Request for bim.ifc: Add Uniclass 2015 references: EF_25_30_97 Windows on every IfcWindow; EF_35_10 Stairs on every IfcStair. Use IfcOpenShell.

First a look at what the model holds.

```python
import ifcopenshell

model = ifcopenshell.open("bim.ifc")
print(model.schema)
print("classifications:", [c.Name for c in model.by_type("IfcClassification")])
for ifc_class in ("IfcDoor", "IfcRoof", "IfcStair", "IfcWall", "IfcWindow"):
    print(ifc_class, len(model.by_type(ifc_class)))
```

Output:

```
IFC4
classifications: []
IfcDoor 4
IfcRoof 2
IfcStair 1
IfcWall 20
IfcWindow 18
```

```python
import ifcopenshell
import ifcopenshell.api.classification

model = ifcopenshell.open("bim.ifc")

system = ifcopenshell.api.classification.add_classification(model, classification="Uniclass 2015")

codes = {
    "IfcWindow": ("EF_25_30_97", "Windows"),
    "IfcStair": ("EF_35_10", "Stairs"),
}
for ifc_class, (code, name) in codes.items():
    products = model.by_type(ifc_class)
    ifcopenshell.api.classification.add_reference(
        model, products=products, classification=system, identification=code, name=name
    )
    print(code, len(products))

model.write("bim_rev.ifc")
```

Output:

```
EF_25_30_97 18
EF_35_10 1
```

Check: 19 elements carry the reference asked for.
